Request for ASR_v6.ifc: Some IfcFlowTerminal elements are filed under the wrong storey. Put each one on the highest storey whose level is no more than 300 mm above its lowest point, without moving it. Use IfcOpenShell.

First a look at what the model holds.

```python
import ifcopenshell
import ifcopenshell.util.element
import ifcopenshell.util.placement

model = ifcopenshell.open("ASR_v6.ifc")
print(model.schema)
for storey in model.by_type("IfcBuildingStorey"):
    level = ifcopenshell.util.placement.get_storey_elevation(storey)
    count = sum(e.is_a("IfcFlowTerminal") for e in ifcopenshell.util.element.get_contained(storey))
    print(storey.id(), storey.Name, round(level, 3), count, sep=" | ")
```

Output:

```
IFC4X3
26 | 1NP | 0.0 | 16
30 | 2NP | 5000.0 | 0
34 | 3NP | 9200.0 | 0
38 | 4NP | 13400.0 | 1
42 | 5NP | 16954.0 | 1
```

```python
import ifcopenshell
import ifcopenshell.api.spatial
import ifcopenshell.geom
import ifcopenshell.util.element
import ifcopenshell.util.placement
import ifcopenshell.util.shape
import ifcopenshell.util.unit

model = ifcopenshell.open("ASR_v6.ifc")
unit_scale = ifcopenshell.util.unit.calculate_unit_scale(model)
settings = ifcopenshell.geom.settings()

levels = sorted(
    ((ifcopenshell.util.placement.get_storey_elevation(s) * unit_scale, s) for s in model.by_type("IfcBuildingStorey")),
    key=lambda pair: pair[0],
)

for e in model.by_type("IfcFlowTerminal"):
    current = e.ContainedInStructure[0].RelatingStructure if e.ContainedInStructure else None
    if current is None or not current.is_a("IfcBuildingStorey"):
        continue
    shape = ifcopenshell.geom.create_shape(settings, e)
    bottom = ifcopenshell.util.shape.get_shape_bottom_elevation(shape, shape.geometry)
    below = [s for level, s in levels if level <= bottom + 0.3]
    storey = below[-1] if below else levels[0][1]
    if storey != current:
        # assign_container keeps the world position.
        ifcopenshell.api.spatial.assign_container(model, products=[e], relating_structure=storey)
        print(e.id(), current.Name, "->", storey.Name)

model.write("ASR_v6_edited.ifc")
```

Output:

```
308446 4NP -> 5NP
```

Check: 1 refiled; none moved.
